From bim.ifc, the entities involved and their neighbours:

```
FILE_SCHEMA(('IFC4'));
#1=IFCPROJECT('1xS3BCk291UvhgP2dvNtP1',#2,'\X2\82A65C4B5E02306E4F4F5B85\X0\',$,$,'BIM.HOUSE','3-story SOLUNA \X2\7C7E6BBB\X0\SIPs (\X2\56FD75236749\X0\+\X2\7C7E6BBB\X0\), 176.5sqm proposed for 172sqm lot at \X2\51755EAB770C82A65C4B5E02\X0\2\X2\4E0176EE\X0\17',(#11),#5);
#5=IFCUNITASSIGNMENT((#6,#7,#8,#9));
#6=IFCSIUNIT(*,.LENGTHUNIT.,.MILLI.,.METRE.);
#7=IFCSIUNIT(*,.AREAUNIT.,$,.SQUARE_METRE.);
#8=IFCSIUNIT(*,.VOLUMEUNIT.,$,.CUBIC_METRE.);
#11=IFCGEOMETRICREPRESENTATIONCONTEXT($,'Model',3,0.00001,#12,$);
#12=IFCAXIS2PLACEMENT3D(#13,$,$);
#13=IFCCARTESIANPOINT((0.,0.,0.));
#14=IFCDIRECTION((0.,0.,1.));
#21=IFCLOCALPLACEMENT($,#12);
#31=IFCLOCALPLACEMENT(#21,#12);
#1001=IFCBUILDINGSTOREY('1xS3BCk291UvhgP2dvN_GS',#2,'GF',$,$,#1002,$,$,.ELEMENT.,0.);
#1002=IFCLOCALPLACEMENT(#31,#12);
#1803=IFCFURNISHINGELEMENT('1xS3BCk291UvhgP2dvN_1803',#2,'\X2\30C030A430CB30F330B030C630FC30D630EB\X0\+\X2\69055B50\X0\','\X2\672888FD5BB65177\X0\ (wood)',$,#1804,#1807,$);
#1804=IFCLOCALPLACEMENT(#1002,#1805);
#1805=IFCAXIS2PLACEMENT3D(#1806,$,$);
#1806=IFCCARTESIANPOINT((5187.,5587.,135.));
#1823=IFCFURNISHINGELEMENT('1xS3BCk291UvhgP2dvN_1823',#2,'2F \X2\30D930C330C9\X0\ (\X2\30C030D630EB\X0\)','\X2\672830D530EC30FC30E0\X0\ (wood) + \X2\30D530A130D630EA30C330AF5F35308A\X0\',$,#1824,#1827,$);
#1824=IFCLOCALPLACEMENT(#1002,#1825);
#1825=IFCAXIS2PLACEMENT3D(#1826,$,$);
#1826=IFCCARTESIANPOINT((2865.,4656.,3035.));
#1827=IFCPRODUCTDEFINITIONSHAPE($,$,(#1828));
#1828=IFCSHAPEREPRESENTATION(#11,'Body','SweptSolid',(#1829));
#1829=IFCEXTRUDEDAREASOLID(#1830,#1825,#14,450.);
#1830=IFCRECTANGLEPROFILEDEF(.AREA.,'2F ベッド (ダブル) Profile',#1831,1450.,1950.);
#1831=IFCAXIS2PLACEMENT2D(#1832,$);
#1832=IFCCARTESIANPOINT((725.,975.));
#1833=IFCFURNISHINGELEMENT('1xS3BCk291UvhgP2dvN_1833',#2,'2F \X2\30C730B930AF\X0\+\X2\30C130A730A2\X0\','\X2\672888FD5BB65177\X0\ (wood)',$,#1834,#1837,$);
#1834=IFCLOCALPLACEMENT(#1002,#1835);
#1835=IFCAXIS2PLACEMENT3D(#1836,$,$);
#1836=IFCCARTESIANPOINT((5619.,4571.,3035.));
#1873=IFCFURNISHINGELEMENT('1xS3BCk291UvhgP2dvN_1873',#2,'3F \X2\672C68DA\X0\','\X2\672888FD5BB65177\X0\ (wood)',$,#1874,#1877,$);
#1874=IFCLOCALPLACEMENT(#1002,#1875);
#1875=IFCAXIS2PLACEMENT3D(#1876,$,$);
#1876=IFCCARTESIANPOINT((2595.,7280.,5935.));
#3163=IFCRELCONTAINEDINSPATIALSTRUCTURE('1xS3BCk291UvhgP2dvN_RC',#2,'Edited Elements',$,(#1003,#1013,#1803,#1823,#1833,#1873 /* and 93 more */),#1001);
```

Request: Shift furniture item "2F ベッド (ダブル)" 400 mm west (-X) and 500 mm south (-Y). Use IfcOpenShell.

```python
import ifcopenshell
import ifcopenshell.api.geometry
import ifcopenshell.util.placement
import ifcopenshell.util.unit

model = ifcopenshell.open("bim.ifc")
unit_scale = ifcopenshell.util.unit.calculate_unit_scale(model)

item = model.by_guid("1xS3BCk291UvhgP2dvN_1823")
matrix = ifcopenshell.util.placement.get_local_placement(item.ObjectPlacement)
matrix[0, 3] -= 0.4 / unit_scale
matrix[1, 3] -= 0.5 / unit_scale
ifcopenshell.api.geometry.edit_object_placement(model, product=item, matrix=matrix, is_si=False)

print(ifcopenshell.util.placement.get_local_placement(item.ObjectPlacement).round(3) + 0.0)

model.write("bim-out.ifc")
```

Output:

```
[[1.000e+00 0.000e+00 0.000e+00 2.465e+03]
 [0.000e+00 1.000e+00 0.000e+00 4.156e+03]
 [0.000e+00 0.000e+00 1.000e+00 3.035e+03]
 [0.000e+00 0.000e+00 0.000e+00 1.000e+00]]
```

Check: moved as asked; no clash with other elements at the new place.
